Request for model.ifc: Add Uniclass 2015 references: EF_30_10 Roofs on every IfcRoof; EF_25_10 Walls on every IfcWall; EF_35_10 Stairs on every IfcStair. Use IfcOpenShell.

First a look at what the model holds.

```python
import ifcopenshell

model = ifcopenshell.open("model.ifc")
print(model.schema)
print("classifications:", [c.Name for c in model.by_type("IfcClassification")])
for ifc_class in ("IfcDoor", "IfcRoof", "IfcStair", "IfcWall", "IfcWindow"):
    print(ifc_class, len(model.by_type(ifc_class)))
```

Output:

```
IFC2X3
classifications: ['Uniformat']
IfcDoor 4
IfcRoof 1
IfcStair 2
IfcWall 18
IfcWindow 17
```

```python
import ifcopenshell
import ifcopenshell.api.classification

model = ifcopenshell.open("model.ifc")

# IFC2X3 requires Source and Edition and has no link from the project to the system.
system = model.create_entity("IfcClassification", Source="NBS", Edition="2015", Name="Uniclass 2015")

codes = {
    "IfcRoof": ("EF_30_10", "Roofs"),
    "IfcWall": ("EF_25_10", "Walls"),
    "IfcStair": ("EF_35_10", "Stairs"),
}
for ifc_class, (code, name) in codes.items():
    products = model.by_type(ifc_class)
    ifcopenshell.api.classification.add_reference(
        model, products=products, classification=system, identification=code, name=name
    )
    print(code, len(products))

model.write("model_edited.ifc")
```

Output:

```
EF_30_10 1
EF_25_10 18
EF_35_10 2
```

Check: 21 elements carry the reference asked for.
